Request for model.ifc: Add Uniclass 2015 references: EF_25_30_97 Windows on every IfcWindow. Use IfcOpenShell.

First a look at what the model holds.

```python
import ifcopenshell

model = ifcopenshell.open("model.ifc")
print(model.schema)
print("classifications:", [c.Name for c in model.by_type("IfcClassification")])
for ifc_class in ("IfcDoor", "IfcRoof", "IfcStair", "IfcWall", "IfcWindow"):
    print(ifc_class, len(model.by_type(ifc_class)))
```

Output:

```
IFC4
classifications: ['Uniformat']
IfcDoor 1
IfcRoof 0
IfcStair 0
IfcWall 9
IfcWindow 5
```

```python
import ifcopenshell
import ifcopenshell.api.classification

model = ifcopenshell.open("model.ifc")

system = ifcopenshell.api.classification.add_classification(model, classification="Uniclass 2015")

codes = {
    "IfcWindow": ("EF_25_30_97", "Windows"),
}
for ifc_class, (code, name) in codes.items():
    products = model.by_type(ifc_class)
    ifcopenshell.api.classification.add_reference(
        model, products=products, classification=system, identification=code, name=name
    )
    print(code, len(products))

model.write("model_v2.ifc")
```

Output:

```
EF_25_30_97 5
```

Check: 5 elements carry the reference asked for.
